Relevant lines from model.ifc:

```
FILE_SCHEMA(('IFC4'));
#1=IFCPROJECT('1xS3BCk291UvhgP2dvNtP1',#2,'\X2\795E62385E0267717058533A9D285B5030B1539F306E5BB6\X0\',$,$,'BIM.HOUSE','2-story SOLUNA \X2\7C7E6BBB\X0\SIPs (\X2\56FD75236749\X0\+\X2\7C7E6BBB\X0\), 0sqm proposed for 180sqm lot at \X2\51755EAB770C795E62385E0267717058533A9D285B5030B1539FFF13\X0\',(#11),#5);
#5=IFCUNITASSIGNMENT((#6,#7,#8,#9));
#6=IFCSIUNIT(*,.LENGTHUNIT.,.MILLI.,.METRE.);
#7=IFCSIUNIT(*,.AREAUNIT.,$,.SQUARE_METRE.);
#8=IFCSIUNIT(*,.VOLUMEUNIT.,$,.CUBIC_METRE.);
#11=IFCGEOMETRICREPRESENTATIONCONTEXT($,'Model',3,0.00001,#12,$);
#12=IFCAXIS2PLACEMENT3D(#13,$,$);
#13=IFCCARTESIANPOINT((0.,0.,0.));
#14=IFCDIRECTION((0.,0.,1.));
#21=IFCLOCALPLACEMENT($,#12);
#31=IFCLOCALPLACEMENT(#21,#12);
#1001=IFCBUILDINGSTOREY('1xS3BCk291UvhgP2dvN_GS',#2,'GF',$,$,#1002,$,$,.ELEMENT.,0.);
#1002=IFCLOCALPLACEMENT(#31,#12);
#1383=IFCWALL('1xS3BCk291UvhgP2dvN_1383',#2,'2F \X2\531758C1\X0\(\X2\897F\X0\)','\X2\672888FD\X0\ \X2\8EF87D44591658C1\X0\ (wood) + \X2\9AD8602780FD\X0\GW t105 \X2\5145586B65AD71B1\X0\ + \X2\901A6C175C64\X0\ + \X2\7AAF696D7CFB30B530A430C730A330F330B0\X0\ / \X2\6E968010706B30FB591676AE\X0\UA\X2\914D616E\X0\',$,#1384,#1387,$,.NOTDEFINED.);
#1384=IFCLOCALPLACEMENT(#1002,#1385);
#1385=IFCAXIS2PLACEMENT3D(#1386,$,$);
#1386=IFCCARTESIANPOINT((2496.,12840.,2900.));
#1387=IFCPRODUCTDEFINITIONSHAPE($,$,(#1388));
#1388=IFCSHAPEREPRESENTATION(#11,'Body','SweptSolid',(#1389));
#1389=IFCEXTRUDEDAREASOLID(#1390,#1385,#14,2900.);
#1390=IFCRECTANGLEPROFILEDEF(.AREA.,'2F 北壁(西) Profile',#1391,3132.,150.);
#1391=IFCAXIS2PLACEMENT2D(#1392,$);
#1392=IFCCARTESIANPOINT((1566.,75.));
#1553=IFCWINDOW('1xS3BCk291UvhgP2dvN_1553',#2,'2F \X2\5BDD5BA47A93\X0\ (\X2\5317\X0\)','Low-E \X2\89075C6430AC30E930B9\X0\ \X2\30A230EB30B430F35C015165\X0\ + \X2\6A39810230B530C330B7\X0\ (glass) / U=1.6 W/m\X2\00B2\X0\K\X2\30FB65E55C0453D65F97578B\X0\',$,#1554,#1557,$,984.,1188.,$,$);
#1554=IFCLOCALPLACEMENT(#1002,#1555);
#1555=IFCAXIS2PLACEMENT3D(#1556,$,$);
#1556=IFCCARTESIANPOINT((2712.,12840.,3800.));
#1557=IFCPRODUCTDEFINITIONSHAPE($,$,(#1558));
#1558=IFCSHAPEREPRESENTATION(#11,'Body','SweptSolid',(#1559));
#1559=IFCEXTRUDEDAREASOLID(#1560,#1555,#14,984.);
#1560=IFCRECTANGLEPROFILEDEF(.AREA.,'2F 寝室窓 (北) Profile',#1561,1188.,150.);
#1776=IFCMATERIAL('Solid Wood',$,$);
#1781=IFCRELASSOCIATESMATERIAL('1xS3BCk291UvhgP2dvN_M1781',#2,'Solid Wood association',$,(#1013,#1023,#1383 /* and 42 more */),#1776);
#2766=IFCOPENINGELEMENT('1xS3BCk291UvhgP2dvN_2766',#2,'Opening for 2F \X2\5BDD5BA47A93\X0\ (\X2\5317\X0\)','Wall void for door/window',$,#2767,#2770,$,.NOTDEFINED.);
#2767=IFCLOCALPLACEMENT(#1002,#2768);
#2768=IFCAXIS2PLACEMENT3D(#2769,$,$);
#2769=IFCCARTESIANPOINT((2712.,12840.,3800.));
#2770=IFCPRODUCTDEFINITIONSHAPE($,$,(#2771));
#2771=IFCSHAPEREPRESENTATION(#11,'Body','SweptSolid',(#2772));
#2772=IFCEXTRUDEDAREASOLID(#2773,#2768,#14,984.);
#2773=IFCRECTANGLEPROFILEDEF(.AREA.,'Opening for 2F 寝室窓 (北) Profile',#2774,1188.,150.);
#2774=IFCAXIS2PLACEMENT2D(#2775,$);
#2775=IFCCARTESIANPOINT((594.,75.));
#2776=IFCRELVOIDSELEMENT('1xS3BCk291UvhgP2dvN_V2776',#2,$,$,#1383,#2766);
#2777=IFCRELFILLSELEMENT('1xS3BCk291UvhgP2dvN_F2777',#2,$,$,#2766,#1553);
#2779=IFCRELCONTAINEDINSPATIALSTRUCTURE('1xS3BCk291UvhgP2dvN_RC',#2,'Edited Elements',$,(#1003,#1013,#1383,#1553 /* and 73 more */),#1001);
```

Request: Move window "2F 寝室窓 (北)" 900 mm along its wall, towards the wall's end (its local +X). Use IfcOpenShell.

```python
import ifcopenshell
import ifcopenshell.api.geometry
import ifcopenshell.util.placement

model = ifcopenshell.open("model.ifc")

window = model.by_guid("1xS3BCk291UvhgP2dvN_1553")
opening = window.FillsVoids[0].RelatingOpeningElement
wall = opening.VoidsElements[0].RelatingBuildingElement

wall_matrix = ifcopenshell.util.placement.get_local_placement(wall.ObjectPlacement)
shift = wall_matrix[:3, 0] * 900.0
before = ifcopenshell.util.placement.get_local_placement(window.ObjectPlacement)[:3, 3].copy()

# The window is not placed relative to its opening, so move both.
for product in (opening, window):
    matrix = ifcopenshell.util.placement.get_local_placement(product.ObjectPlacement)
    matrix[:3, 3] += shift
    ifcopenshell.api.geometry.edit_object_placement(model, product=product, matrix=matrix, is_si=False)

after = ifcopenshell.util.placement.get_local_placement(window.ObjectPlacement)[:3, 3]
print("window moved by", (after - before).round(3) + 0.0)

model.write("model_updated.ifc")
```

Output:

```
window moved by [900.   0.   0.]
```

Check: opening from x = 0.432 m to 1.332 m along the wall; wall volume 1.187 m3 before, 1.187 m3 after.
